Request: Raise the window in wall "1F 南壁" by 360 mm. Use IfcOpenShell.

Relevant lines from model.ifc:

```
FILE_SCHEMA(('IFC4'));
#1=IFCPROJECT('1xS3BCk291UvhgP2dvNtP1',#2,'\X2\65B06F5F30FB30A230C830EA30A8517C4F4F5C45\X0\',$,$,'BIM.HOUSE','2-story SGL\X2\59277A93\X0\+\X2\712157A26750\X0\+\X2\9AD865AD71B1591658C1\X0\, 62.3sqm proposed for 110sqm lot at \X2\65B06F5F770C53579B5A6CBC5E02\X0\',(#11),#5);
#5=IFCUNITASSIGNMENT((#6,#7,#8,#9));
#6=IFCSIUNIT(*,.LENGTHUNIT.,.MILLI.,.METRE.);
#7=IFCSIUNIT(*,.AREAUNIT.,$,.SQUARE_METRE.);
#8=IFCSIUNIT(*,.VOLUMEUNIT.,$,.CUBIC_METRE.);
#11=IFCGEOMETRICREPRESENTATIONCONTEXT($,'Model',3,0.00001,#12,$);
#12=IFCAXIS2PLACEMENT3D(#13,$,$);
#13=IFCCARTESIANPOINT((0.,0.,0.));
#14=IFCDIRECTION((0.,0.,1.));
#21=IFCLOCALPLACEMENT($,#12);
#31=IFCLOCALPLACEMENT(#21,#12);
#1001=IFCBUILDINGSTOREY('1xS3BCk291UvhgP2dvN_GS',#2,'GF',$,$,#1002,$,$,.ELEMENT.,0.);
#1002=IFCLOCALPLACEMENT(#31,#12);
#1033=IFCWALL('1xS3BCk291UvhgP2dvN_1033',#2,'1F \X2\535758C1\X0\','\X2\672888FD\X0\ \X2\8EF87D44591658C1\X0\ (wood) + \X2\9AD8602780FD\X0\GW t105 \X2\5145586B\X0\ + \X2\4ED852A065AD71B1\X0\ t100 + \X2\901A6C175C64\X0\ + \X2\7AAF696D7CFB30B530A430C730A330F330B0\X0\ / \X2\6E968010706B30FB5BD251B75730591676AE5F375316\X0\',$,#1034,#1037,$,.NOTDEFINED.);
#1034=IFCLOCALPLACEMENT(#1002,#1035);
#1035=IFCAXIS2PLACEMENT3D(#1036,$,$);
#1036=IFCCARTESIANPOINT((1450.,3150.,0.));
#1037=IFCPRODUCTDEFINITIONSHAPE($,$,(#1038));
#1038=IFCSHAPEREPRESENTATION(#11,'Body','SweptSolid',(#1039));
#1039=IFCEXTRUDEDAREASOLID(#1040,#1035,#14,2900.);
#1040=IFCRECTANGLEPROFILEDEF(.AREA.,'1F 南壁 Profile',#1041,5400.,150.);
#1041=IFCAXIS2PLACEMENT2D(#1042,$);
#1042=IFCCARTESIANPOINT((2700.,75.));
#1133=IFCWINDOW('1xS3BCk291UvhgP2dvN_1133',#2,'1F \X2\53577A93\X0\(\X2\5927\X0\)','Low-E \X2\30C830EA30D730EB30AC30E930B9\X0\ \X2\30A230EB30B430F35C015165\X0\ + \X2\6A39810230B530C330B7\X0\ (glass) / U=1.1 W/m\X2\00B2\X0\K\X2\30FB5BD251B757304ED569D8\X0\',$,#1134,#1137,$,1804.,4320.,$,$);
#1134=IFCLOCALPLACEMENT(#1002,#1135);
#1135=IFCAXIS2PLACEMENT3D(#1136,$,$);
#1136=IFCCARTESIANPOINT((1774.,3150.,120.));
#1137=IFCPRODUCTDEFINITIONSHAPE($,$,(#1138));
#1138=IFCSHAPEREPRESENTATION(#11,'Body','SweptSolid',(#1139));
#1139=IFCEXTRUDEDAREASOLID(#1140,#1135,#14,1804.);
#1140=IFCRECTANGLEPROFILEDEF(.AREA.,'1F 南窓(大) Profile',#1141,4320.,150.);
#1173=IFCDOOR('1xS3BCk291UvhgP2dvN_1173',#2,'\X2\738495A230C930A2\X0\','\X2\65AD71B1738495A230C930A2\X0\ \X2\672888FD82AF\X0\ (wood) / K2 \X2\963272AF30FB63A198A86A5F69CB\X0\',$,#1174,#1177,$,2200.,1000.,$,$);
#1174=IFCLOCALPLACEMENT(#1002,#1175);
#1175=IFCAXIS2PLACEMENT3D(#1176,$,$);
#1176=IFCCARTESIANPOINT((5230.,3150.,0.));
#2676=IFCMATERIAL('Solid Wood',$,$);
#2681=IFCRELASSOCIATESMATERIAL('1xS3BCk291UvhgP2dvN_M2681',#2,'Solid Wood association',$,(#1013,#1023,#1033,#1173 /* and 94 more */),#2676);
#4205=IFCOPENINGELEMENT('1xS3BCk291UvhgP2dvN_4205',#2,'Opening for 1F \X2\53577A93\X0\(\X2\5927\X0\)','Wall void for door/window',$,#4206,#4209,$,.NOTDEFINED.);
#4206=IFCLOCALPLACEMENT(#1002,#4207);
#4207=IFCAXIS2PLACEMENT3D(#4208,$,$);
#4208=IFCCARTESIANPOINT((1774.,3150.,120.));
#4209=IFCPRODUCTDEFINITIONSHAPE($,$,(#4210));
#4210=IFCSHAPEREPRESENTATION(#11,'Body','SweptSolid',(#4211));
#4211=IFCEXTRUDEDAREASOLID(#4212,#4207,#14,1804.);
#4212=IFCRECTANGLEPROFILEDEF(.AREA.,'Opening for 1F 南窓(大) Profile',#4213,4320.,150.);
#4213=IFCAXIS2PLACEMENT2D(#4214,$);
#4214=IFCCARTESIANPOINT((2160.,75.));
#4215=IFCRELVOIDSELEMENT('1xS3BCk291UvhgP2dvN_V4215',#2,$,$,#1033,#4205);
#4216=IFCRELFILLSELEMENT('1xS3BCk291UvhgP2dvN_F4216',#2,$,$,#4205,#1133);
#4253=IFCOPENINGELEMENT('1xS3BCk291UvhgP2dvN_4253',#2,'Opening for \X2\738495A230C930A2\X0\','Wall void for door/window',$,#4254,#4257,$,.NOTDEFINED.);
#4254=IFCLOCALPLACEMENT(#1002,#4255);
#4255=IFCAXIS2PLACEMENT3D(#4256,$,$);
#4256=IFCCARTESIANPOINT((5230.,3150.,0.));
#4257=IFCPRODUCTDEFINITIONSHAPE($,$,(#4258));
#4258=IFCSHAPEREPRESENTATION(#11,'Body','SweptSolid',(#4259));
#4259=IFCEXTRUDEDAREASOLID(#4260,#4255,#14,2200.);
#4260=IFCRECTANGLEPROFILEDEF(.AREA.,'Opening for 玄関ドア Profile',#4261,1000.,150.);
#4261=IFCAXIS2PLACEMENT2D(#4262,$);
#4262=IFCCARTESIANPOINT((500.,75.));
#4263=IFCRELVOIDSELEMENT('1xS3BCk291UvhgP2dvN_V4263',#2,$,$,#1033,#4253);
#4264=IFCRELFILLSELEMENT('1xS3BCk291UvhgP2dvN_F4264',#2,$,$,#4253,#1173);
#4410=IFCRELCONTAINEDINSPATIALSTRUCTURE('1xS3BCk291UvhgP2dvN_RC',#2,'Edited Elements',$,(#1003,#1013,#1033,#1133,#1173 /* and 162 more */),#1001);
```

```python
import numpy as np
import ifcopenshell
import ifcopenshell.api.geometry
import ifcopenshell.util.placement
import ifcopenshell.util.unit

model = ifcopenshell.open("model.ifc")
unit_scale = ifcopenshell.util.unit.calculate_unit_scale(model)

window = model.by_guid("1xS3BCk291UvhgP2dvN_1133")
opening = window.FillsVoids[0].RelatingOpeningElement
dz = 360.0

shift = np.array([0.0, 0.0, dz])
# The window is not placed relative to its opening, so move both.
for product in (opening, window):
    matrix = ifcopenshell.util.placement.get_local_placement(product.ObjectPlacement)
    matrix[:3, 3] += shift
    ifcopenshell.api.geometry.edit_object_placement(model, product=product, matrix=matrix, is_si=False)

print(f"moved by {dz * unit_scale:+.3f} m")

model.write("model_rev.ifc")
```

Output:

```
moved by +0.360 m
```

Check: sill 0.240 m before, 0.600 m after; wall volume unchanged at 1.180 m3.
